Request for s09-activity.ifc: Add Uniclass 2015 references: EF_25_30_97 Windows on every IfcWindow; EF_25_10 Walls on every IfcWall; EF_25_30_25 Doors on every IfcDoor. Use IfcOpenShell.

First a look at what the model holds.

```python
import ifcopenshell

model = ifcopenshell.open("s09-activity.ifc")
print(model.schema)
print("classifications:", [c.Name for c in model.by_type("IfcClassification")])
for ifc_class in ("IfcDoor", "IfcRoof", "IfcStair", "IfcWall", "IfcWindow"):
    print(ifc_class, len(model.by_type(ifc_class)))
```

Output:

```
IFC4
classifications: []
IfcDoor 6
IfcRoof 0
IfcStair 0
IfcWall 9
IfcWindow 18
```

```python
import ifcopenshell
import ifcopenshell.api.classification

model = ifcopenshell.open("s09-activity.ifc")

system = ifcopenshell.api.classification.add_classification(model, classification="Uniclass 2015")

codes = {
    "IfcWindow": ("EF_25_30_97", "Windows"),
    "IfcWall": ("EF_25_10", "Walls"),
    "IfcDoor": ("EF_25_30_25", "Doors"),
}
for ifc_class, (code, name) in codes.items():
    products = model.by_type(ifc_class)
    ifcopenshell.api.classification.add_reference(
        model, products=products, classification=system, identification=code, name=name
    )
    print(code, len(products))

model.write("s09-activity_updated.ifc")
```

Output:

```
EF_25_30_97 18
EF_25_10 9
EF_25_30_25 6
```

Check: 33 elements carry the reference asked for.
